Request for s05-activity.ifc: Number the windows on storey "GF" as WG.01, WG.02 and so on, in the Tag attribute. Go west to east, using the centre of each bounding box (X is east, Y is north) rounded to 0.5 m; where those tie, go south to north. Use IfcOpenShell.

First a look at what the model holds.

```python
import ifcopenshell
import ifcopenshell.util.element
import ifcopenshell.util.placement

model = ifcopenshell.open("s05-activity.ifc")
print(model.schema)
storey = next(s for s in model.by_type("IfcBuildingStorey") if s.Name == "GF")
windows = [e for e in ifcopenshell.util.element.get_decomposition(storey) if e.is_a("IfcWindow")]
for e in sorted(windows, key=lambda e: e.id()):
    origin = ifcopenshell.util.placement.get_local_placement(e.ObjectPlacement)[:3, 3]
    print(e.id(), e.Tag, e.Name, origin.round(2) + 0.0, sep=" | ")
```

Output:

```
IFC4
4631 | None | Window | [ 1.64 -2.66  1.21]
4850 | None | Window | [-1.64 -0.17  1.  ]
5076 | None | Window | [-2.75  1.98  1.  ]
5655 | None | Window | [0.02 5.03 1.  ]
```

```python
import ifcopenshell
import ifcopenshell.geom
import ifcopenshell.util.element
import ifcopenshell.util.shape

model = ifcopenshell.open("s05-activity.ifc")
settings = ifcopenshell.geom.settings()
settings.set("use-world-coords", True)


def centre(element):
    shape = ifcopenshell.geom.create_shape(settings, element)
    return ifcopenshell.util.shape.get_bbox_centroid(shape.geometry)


storey = next(s for s in model.by_type("IfcBuildingStorey") if s.Name == "GF")
windows = [e for e in ifcopenshell.util.element.get_decomposition(storey) if e.is_a("IfcWindow")]

# Insertion points can sit at a corner or the storey origin, so sort by the geometry (in metres).
centres = {e: centre(e) for e in windows}
windows.sort(key=lambda e: (round(centres[e][0] / 0.5), centres[e][1]))

for i, e in enumerate(windows, start=1):
    number = f"WG.{i:02d}"
    e.Tag = number
    print(e.id(), number)

model.write("s05-activity_edited.ifc")
```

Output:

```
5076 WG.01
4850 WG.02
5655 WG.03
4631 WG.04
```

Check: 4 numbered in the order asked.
